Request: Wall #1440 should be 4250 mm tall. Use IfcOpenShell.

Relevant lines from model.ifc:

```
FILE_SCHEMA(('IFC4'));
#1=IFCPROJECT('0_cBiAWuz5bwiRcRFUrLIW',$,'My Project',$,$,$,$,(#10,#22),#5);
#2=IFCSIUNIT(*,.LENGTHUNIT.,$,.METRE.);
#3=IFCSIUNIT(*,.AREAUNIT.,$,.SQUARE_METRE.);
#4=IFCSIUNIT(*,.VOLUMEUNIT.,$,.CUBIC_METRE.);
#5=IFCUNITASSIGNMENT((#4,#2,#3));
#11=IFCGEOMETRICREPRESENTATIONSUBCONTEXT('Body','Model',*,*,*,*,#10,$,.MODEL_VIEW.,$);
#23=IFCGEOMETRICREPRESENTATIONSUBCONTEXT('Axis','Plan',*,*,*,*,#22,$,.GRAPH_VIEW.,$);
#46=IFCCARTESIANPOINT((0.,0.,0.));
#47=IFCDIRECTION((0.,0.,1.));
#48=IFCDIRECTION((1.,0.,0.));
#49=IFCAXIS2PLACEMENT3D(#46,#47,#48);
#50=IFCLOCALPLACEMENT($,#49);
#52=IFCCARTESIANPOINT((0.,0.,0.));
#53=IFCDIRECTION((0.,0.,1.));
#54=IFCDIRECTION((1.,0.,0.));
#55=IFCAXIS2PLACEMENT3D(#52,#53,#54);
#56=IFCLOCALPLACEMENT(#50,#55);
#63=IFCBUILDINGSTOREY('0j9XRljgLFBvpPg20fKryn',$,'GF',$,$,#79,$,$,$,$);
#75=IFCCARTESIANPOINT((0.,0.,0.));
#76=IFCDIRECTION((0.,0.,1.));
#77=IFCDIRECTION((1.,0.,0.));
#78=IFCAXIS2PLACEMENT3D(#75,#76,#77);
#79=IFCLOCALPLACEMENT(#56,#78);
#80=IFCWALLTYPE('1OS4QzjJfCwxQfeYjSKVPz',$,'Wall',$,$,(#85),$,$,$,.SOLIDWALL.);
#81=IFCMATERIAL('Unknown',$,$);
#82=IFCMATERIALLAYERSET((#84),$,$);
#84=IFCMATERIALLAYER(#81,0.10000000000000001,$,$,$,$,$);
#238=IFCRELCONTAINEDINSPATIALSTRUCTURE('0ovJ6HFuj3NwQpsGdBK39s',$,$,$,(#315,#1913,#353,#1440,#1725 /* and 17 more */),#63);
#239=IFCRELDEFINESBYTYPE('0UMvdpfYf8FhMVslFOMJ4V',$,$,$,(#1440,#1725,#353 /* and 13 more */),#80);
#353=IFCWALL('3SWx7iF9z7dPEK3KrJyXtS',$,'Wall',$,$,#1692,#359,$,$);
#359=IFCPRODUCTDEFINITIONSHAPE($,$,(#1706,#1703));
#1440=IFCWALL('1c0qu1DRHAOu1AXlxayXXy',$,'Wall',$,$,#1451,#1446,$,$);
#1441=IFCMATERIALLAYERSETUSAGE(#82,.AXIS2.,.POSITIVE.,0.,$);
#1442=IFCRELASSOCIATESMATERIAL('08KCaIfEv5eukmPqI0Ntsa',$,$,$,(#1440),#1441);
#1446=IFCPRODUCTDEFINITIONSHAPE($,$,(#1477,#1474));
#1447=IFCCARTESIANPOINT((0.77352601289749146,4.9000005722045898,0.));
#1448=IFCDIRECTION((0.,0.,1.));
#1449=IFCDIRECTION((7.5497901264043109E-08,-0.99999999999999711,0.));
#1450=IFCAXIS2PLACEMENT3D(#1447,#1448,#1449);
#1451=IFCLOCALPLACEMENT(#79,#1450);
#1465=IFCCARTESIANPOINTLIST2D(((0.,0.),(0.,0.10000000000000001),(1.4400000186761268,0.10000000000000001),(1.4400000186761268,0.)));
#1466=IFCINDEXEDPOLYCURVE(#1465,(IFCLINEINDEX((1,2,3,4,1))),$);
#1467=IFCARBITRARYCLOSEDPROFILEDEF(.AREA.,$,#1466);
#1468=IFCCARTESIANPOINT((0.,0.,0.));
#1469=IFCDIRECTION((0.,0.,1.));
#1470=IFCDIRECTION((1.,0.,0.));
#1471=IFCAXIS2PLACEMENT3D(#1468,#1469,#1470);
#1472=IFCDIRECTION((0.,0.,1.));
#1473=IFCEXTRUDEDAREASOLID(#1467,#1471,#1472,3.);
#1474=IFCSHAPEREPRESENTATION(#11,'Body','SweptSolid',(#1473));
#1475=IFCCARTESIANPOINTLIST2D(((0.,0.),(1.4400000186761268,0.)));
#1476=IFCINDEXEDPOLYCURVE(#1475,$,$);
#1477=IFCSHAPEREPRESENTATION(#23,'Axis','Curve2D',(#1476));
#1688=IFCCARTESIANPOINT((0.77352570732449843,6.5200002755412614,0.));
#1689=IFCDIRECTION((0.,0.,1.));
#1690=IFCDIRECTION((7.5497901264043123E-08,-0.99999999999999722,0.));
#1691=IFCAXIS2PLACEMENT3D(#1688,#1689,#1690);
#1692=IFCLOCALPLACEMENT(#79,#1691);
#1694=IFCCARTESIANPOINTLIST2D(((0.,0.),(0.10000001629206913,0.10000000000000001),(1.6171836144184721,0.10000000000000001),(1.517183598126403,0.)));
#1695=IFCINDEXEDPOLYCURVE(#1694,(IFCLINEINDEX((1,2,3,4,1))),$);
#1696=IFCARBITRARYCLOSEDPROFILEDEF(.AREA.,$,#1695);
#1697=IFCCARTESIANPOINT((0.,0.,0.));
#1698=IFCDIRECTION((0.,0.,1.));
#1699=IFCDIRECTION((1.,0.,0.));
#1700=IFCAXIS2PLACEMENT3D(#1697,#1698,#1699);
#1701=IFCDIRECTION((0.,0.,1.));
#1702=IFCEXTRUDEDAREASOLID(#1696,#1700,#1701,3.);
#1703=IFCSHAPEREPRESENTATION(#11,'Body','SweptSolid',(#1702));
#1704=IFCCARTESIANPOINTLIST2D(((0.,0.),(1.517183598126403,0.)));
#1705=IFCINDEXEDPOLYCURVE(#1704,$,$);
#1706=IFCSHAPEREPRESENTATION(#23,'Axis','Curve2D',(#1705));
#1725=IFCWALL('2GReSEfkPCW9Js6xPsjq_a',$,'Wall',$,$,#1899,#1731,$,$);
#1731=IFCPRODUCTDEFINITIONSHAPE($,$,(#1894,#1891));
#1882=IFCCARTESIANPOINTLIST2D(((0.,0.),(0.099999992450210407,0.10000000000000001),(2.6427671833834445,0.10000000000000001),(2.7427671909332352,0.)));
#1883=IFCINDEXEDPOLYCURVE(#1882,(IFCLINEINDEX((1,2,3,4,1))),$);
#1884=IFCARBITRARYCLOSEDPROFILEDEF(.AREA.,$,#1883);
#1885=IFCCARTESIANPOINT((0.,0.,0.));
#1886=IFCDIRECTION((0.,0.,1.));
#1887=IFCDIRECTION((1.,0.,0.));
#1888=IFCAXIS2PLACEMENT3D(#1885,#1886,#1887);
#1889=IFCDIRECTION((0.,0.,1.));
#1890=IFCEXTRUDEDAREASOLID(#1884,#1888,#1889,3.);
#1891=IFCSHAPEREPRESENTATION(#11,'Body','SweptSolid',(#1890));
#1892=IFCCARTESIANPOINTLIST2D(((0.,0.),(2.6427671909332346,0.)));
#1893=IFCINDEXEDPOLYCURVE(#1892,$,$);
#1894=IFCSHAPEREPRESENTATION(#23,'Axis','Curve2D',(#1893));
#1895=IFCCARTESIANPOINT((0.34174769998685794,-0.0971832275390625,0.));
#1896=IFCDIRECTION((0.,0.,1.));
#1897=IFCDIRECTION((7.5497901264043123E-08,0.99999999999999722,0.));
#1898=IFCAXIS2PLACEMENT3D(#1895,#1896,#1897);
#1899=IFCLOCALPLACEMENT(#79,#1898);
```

```python
import ifcopenshell
import ifcopenshell.geom
import ifcopenshell.util.representation
import ifcopenshell.util.shape
import ifcopenshell.util.unit

model = ifcopenshell.open("model.ifc")
unit_scale = ifcopenshell.util.unit.calculate_unit_scale(model)
settings = ifcopenshell.geom.settings()


def volume(element):
    """Net volume in cubic metres, openings subtracted."""
    shape = ifcopenshell.geom.create_shape(settings, element)
    return ifcopenshell.util.shape.get_volume(shape.geometry)


wall = model.by_guid("1c0qu1DRHAOu1AXlxayXXy")
before = volume(wall)

body = ifcopenshell.util.representation.get_representation(wall, "Model", "Body")
solid = body.Items[0]
old_height = solid.Depth
solid.Depth = 4.25 / unit_scale
after = volume(wall)

print(f"height {old_height:g} -> {solid.Depth:g}, volume {before:.3f} -> {after:.3f} m3")

model.write("model_rev.ifc")
```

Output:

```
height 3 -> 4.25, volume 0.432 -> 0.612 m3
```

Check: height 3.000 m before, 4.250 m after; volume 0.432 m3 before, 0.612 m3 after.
